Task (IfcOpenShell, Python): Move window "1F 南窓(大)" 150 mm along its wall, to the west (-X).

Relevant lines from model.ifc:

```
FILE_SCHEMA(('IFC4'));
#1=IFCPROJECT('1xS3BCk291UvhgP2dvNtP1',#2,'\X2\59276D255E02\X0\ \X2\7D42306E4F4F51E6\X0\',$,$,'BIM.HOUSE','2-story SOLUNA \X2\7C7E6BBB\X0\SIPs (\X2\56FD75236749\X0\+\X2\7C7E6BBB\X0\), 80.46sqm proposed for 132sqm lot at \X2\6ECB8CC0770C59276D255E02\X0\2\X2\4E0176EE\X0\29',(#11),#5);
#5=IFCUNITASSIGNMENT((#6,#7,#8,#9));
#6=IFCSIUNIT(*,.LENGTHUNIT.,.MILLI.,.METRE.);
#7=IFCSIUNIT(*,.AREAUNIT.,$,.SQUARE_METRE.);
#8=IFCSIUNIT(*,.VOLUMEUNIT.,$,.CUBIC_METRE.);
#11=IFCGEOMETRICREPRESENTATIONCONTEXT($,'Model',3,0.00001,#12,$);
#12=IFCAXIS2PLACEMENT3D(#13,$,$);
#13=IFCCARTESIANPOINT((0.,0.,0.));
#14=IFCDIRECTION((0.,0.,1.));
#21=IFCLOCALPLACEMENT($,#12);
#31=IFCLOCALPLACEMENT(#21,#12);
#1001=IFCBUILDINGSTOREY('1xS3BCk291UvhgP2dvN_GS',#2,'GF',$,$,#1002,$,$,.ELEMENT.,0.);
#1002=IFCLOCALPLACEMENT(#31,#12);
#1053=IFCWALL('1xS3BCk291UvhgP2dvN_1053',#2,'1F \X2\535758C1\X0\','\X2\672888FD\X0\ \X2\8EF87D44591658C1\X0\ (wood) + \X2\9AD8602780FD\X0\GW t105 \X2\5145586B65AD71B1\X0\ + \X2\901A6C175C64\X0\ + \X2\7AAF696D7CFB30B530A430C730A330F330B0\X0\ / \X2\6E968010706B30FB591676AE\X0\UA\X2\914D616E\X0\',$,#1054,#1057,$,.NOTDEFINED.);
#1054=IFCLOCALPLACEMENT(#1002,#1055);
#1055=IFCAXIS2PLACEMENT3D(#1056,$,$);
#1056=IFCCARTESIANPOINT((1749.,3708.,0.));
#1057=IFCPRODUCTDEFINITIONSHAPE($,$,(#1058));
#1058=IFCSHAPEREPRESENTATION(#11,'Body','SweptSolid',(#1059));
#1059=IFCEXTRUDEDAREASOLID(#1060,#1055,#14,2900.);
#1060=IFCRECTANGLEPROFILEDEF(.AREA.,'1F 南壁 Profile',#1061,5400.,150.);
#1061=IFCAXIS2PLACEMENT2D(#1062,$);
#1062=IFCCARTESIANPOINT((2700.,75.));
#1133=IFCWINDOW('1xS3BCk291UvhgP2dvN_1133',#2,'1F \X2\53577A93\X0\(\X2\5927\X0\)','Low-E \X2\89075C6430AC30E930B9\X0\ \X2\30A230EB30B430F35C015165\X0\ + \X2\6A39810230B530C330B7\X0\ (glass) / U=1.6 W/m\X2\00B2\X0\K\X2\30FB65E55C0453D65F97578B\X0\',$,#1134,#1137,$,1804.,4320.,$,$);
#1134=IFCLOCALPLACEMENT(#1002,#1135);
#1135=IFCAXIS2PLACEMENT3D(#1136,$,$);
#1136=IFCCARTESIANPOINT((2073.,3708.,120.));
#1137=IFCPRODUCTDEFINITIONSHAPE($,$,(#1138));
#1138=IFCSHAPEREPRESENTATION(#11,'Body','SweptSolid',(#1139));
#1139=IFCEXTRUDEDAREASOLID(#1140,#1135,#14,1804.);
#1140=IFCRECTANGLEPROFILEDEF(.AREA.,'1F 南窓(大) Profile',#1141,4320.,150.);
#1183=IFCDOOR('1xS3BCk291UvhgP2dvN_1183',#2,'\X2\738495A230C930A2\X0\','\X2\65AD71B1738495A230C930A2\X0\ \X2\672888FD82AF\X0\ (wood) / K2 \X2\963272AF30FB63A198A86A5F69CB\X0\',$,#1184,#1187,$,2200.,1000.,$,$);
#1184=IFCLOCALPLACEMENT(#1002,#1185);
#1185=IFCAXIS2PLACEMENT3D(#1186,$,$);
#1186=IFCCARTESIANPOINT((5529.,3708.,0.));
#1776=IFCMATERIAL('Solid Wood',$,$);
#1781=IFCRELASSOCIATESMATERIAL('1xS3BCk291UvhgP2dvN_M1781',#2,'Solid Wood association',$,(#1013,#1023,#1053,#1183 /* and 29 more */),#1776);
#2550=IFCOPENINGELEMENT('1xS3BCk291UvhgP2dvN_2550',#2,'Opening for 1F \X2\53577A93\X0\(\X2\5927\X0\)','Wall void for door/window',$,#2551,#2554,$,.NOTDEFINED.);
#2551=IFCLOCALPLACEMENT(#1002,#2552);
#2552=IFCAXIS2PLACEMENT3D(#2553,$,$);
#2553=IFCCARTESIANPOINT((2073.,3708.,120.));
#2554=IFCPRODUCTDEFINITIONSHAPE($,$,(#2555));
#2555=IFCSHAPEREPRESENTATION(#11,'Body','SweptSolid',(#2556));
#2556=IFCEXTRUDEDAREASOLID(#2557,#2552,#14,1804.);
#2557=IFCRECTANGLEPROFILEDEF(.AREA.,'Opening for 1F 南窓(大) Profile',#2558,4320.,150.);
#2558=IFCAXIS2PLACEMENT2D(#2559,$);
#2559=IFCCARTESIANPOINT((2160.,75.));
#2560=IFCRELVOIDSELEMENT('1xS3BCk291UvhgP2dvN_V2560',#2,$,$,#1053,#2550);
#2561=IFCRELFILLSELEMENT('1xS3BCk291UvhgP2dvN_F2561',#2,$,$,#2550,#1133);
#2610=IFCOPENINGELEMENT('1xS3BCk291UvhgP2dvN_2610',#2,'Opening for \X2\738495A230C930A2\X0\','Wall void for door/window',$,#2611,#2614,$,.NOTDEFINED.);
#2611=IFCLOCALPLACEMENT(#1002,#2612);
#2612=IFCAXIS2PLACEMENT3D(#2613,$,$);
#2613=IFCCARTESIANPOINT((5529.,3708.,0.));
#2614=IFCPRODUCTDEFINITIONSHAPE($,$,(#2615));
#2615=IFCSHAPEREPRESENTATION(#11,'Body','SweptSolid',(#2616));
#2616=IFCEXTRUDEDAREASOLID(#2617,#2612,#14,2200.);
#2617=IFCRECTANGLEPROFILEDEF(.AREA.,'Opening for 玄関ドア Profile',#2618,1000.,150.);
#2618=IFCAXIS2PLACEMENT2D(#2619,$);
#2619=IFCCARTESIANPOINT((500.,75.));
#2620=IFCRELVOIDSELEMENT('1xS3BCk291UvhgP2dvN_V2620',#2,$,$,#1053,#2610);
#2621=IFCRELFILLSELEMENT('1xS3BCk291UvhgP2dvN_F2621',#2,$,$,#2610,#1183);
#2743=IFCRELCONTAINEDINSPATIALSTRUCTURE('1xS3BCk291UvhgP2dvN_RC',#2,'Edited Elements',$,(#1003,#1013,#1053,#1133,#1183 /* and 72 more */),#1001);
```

```python
import ifcopenshell
import ifcopenshell.api.geometry
import ifcopenshell.util.placement

model = ifcopenshell.open("model.ifc")

window = model.by_id(1133)
opening = window.FillsVoids[0].RelatingOpeningElement
wall = opening.VoidsElements[0].RelatingBuildingElement

wall_matrix = ifcopenshell.util.placement.get_local_placement(wall.ObjectPlacement)
shift = wall_matrix[:3, 0] * -150.0
before = ifcopenshell.util.placement.get_local_placement(window.ObjectPlacement)[:3, 3].copy()

# The window is not placed relative to its opening, so move both.
for product in (opening, window):
    matrix = ifcopenshell.util.placement.get_local_placement(product.ObjectPlacement)
    matrix[:3, 3] += shift
    ifcopenshell.api.geometry.edit_object_placement(model, product=product, matrix=matrix, is_si=False)

after = ifcopenshell.util.placement.get_local_placement(window.ObjectPlacement)[:3, 3]
print("window moved by", (after - before).round(3) + 0.0)

model.write("model-out.ifc")
```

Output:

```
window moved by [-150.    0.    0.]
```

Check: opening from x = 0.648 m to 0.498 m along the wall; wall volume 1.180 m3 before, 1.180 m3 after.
